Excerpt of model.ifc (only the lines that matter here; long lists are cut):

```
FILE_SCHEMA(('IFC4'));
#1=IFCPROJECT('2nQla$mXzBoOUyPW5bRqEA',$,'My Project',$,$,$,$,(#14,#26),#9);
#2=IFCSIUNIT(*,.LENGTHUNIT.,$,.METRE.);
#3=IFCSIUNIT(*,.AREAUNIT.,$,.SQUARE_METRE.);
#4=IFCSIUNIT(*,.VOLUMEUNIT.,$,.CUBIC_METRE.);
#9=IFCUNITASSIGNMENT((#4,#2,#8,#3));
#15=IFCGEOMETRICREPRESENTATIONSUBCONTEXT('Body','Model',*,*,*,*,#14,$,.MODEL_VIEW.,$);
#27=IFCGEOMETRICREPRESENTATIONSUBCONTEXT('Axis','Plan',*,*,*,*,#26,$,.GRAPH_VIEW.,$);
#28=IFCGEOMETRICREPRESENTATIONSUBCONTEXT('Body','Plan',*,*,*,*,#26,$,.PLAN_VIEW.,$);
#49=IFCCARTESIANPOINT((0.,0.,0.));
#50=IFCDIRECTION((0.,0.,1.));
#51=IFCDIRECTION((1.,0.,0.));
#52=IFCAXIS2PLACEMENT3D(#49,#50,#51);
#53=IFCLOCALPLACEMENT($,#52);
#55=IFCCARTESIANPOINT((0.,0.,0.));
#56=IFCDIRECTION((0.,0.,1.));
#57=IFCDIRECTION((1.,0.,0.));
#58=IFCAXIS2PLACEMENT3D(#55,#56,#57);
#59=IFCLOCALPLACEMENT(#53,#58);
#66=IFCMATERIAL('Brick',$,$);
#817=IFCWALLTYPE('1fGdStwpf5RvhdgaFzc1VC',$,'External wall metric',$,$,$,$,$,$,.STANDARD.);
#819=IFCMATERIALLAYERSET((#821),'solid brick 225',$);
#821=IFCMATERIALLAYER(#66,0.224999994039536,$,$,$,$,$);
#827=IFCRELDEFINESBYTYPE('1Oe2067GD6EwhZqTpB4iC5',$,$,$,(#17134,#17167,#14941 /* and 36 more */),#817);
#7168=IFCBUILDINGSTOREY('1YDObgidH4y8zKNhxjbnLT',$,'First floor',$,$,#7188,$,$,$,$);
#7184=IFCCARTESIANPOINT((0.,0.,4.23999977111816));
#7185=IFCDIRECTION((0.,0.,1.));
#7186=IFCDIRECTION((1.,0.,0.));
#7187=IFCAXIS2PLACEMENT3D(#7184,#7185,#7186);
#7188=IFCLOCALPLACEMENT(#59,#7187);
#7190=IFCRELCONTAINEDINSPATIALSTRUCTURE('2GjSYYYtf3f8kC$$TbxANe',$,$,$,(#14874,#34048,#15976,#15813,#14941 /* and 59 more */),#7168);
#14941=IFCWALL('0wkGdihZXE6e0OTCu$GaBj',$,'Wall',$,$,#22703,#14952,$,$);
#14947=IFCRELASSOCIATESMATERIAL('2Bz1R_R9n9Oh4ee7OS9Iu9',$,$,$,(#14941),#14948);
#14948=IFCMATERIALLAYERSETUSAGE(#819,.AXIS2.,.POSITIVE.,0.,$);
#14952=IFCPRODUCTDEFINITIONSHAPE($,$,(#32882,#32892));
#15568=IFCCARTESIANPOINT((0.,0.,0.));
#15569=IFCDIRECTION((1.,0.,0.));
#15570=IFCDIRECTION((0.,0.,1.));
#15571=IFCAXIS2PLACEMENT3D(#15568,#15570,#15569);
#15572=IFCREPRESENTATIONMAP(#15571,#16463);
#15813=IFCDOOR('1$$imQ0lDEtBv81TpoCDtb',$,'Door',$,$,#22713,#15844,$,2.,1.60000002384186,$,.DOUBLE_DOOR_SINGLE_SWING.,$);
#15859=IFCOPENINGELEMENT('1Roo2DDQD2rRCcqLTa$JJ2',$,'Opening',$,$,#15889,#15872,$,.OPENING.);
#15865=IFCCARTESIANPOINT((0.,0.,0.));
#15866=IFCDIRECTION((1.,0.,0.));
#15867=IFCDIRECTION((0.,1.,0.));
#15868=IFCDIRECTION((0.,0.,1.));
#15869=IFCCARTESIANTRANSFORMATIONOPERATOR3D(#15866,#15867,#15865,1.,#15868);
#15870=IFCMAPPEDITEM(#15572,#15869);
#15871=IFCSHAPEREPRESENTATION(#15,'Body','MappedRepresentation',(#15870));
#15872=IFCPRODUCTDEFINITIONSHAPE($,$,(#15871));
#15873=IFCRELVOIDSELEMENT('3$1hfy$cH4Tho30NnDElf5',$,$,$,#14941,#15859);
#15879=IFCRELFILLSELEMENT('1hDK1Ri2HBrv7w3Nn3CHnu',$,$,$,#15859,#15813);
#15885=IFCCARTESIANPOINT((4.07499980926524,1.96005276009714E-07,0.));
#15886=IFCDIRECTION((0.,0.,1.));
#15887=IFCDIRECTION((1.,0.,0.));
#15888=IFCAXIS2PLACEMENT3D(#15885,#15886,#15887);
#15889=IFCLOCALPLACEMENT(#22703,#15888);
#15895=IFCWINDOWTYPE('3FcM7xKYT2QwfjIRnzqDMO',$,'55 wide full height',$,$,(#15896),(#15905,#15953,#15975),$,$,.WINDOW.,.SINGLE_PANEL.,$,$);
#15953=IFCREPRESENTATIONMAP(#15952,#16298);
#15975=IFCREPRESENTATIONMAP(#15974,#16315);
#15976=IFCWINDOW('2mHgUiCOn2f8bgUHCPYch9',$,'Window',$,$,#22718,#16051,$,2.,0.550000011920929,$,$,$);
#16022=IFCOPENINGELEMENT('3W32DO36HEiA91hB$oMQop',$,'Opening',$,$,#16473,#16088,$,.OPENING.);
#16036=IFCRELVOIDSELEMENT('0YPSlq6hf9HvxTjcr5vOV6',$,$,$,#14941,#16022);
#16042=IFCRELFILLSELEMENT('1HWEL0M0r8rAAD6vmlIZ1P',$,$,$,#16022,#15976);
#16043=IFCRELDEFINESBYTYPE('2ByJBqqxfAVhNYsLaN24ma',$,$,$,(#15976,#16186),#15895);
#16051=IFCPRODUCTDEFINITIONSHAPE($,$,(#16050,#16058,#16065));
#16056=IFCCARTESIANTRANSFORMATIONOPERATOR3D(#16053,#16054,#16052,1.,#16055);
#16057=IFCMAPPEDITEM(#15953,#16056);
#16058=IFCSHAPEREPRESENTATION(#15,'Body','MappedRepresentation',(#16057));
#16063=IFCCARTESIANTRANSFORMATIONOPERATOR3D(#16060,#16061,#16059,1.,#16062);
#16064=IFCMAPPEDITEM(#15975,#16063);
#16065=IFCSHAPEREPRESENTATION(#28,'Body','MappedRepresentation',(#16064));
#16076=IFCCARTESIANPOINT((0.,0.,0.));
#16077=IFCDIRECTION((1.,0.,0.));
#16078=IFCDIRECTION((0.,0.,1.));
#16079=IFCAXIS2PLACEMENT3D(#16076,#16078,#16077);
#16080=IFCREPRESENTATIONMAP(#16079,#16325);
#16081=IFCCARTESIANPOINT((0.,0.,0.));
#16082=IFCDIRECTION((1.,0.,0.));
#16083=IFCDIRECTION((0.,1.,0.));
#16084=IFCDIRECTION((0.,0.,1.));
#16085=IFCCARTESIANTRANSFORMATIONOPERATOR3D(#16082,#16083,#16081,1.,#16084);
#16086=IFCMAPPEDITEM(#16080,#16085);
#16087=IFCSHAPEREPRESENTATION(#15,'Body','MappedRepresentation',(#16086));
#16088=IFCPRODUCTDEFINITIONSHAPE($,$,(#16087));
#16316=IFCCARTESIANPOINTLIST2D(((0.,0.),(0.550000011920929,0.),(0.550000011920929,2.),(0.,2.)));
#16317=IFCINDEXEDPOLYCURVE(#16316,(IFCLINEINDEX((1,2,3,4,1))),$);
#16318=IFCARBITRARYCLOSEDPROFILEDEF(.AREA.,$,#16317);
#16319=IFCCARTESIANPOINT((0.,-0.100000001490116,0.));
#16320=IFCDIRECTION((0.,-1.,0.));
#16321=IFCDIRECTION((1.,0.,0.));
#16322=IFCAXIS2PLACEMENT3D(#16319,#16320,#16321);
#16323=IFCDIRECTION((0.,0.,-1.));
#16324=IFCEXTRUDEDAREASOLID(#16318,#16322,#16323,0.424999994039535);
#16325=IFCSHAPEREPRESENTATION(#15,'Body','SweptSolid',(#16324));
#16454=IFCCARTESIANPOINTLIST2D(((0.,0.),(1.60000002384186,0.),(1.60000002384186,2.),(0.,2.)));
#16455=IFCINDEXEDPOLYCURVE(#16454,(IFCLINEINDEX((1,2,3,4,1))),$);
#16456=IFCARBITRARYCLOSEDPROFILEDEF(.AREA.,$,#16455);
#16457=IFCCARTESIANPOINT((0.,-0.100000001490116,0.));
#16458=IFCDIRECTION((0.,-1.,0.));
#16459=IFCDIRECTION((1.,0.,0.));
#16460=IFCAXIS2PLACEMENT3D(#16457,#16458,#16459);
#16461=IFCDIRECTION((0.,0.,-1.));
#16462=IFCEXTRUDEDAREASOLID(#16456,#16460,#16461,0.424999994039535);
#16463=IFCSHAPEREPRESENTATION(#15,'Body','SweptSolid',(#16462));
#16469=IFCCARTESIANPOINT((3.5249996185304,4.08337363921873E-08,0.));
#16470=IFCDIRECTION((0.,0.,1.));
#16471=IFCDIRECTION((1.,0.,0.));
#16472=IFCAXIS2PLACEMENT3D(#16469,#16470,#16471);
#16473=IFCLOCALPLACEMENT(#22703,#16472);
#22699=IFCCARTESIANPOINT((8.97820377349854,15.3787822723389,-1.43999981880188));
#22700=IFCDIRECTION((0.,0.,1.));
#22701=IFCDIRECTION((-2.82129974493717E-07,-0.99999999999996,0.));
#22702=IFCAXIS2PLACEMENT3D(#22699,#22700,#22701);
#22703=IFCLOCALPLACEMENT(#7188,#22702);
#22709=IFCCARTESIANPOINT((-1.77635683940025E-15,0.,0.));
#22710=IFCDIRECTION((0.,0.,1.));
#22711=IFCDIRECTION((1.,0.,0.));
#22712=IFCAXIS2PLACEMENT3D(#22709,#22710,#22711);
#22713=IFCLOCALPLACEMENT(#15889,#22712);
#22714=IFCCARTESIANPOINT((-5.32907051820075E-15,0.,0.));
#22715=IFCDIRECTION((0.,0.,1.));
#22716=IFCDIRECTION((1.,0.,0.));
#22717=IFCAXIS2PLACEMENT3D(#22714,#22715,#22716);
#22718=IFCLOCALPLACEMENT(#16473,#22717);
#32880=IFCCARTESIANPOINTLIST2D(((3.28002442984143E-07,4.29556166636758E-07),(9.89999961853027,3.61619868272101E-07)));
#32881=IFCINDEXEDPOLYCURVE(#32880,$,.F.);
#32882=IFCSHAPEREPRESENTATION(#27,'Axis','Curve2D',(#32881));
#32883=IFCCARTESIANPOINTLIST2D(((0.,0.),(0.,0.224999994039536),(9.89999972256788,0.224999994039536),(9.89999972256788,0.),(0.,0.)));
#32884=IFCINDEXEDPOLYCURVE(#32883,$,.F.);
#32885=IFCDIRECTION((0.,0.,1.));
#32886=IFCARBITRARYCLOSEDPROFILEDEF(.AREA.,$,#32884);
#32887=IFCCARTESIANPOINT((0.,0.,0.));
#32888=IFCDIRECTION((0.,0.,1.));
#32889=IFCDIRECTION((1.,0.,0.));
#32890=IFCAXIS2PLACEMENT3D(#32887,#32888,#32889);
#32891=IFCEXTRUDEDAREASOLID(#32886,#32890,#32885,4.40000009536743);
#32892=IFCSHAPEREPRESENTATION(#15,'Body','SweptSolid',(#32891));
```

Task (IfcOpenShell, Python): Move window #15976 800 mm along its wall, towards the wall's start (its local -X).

```python
import ifcopenshell
import ifcopenshell.api.geometry
import ifcopenshell.util.placement

model = ifcopenshell.open("model.ifc")

window = model.by_guid("2mHgUiCOn2f8bgUHCPYch9")
opening = window.FillsVoids[0].RelatingOpeningElement
wall = opening.VoidsElements[0].RelatingBuildingElement

wall_matrix = ifcopenshell.util.placement.get_local_placement(wall.ObjectPlacement)
shift = wall_matrix[:3, 0] * -0.8
before = ifcopenshell.util.placement.get_local_placement(window.ObjectPlacement)[:3, 3].copy()

# The window is placed relative to its opening, so it follows when the opening moves.
matrix = ifcopenshell.util.placement.get_local_placement(opening.ObjectPlacement)
matrix[:3, 3] += shift
ifcopenshell.api.geometry.edit_object_placement(
    model, product=opening, matrix=matrix, is_si=False, should_transform_children=True
)

after = ifcopenshell.util.placement.get_local_placement(window.ObjectPlacement)[:3, 3]
print("window moved by", (after - before).round(3) + 0.0)

model.write("model-out.ifc")
```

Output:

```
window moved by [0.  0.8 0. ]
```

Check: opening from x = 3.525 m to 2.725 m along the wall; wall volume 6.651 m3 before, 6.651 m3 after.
